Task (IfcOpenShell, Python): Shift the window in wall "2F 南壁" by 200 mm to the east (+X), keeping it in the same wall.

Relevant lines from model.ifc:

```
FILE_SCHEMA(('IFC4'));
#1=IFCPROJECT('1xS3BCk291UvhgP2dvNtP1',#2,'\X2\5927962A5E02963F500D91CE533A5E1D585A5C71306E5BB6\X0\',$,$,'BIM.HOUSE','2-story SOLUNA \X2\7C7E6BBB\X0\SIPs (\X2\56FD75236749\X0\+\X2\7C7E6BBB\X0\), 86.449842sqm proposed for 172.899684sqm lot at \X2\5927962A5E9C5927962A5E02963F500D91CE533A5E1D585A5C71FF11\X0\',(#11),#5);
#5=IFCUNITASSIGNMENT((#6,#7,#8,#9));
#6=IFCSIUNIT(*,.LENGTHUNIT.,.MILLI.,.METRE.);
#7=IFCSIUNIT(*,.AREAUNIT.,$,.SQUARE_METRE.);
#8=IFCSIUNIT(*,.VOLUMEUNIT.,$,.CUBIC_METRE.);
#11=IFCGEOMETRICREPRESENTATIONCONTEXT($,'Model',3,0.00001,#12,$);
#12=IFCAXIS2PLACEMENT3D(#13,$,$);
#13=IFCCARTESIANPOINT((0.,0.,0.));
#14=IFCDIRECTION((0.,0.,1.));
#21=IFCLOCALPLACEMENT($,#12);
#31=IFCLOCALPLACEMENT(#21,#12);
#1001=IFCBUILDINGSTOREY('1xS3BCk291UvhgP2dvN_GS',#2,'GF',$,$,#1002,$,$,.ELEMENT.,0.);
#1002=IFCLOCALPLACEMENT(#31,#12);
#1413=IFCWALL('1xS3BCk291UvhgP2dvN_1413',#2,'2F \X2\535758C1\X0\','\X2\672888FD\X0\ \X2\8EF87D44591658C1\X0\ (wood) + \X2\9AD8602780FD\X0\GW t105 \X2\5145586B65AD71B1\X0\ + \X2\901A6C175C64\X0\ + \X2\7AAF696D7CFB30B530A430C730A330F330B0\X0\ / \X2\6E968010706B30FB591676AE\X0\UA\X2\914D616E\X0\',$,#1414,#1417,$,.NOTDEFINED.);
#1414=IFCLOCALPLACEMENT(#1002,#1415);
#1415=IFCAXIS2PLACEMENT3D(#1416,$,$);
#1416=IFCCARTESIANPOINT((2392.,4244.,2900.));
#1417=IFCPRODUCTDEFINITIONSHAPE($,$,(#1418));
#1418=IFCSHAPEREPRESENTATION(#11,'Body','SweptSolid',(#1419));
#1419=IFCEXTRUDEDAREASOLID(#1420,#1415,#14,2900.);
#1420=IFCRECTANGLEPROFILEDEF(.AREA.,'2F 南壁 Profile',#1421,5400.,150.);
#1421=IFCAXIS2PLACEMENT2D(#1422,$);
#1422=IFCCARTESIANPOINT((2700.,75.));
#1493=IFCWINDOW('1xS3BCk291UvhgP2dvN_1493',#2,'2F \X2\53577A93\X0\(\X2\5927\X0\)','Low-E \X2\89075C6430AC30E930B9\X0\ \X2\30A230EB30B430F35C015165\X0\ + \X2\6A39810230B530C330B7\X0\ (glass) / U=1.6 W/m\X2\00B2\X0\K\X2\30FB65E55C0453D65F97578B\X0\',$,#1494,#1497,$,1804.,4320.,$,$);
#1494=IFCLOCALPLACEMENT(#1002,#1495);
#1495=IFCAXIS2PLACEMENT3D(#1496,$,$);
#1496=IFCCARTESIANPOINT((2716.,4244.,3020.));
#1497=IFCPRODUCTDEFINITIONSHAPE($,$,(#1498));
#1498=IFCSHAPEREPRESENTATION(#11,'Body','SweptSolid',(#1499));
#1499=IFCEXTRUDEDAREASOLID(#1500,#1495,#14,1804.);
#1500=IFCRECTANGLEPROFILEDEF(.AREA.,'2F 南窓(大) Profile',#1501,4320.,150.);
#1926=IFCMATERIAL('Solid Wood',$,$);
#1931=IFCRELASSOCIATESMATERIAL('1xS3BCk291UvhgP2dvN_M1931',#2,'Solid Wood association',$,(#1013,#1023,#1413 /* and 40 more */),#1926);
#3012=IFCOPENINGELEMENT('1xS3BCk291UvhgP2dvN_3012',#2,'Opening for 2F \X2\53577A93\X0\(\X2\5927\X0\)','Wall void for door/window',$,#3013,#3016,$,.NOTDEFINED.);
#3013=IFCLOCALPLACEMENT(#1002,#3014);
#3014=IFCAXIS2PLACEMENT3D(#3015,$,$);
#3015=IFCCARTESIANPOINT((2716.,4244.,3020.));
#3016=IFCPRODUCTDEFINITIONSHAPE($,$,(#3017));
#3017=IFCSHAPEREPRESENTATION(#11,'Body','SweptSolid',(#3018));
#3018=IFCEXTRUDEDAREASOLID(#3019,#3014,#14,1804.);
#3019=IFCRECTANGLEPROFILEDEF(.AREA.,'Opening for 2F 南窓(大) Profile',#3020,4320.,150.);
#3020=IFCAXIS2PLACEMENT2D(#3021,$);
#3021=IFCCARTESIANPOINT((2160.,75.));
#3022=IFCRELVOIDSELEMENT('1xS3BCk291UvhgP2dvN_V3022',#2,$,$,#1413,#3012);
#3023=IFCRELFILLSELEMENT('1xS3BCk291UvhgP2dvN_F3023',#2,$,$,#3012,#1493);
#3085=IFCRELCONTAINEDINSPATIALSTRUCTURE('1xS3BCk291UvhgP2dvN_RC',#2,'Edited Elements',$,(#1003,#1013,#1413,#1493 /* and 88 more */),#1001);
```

```python
import ifcopenshell
import ifcopenshell.api.geometry
import ifcopenshell.util.placement
import ifcopenshell.util.unit

model = ifcopenshell.open("model.ifc")
unit_scale = ifcopenshell.util.unit.calculate_unit_scale(model)

window = model.by_guid("1xS3BCk291UvhgP2dvN_1493")
opening = window.FillsVoids[0].RelatingOpeningElement
wall = opening.VoidsElements[0].RelatingBuildingElement

wall_matrix = ifcopenshell.util.placement.get_local_placement(wall.ObjectPlacement)
shift = wall_matrix[:3, 0] * 0.2 / unit_scale
before = ifcopenshell.util.placement.get_local_placement(window.ObjectPlacement)[:3, 3].copy()

# The window is not placed relative to its opening, so move both.
for product in (opening, window):
    matrix = ifcopenshell.util.placement.get_local_placement(product.ObjectPlacement)
    matrix[:3, 3] += shift
    ifcopenshell.api.geometry.edit_object_placement(model, product=product, matrix=matrix, is_si=False)

after = ifcopenshell.util.placement.get_local_placement(window.ObjectPlacement)[:3, 3]
print("window moved by", (after - before).round(3) + 0.0)

model.write("model-out.ifc")
```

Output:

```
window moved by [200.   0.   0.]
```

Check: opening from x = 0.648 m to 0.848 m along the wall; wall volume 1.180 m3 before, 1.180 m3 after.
